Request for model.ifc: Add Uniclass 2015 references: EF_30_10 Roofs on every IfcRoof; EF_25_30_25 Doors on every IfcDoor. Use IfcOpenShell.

First a look at what the model holds.

```python
import ifcopenshell

model = ifcopenshell.open("model.ifc")
print(model.schema)
print("classifications:", [c.Name for c in model.by_type("IfcClassification")])
for ifc_class in ("IfcDoor", "IfcRoof", "IfcStair", "IfcWall", "IfcWindow"):
    print(ifc_class, len(model.by_type(ifc_class)))
```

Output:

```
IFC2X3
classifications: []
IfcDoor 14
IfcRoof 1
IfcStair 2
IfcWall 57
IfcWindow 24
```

```python
import ifcopenshell
import ifcopenshell.api.classification

model = ifcopenshell.open("model.ifc")

# IFC2X3 requires Source and Edition and has no link from the project to the system.
system = model.create_entity("IfcClassification", Source="NBS", Edition="2015", Name="Uniclass 2015")

codes = {
    "IfcRoof": ("EF_30_10", "Roofs"),
    "IfcDoor": ("EF_25_30_25", "Doors"),
}
for ifc_class, (code, name) in codes.items():
    products = model.by_type(ifc_class)
    ifcopenshell.api.classification.add_reference(
        model, products=products, classification=system, identification=code, name=name
    )
    print(code, len(products))

model.write("model_rev.ifc")
```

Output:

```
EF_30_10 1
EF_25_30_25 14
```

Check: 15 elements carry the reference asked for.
